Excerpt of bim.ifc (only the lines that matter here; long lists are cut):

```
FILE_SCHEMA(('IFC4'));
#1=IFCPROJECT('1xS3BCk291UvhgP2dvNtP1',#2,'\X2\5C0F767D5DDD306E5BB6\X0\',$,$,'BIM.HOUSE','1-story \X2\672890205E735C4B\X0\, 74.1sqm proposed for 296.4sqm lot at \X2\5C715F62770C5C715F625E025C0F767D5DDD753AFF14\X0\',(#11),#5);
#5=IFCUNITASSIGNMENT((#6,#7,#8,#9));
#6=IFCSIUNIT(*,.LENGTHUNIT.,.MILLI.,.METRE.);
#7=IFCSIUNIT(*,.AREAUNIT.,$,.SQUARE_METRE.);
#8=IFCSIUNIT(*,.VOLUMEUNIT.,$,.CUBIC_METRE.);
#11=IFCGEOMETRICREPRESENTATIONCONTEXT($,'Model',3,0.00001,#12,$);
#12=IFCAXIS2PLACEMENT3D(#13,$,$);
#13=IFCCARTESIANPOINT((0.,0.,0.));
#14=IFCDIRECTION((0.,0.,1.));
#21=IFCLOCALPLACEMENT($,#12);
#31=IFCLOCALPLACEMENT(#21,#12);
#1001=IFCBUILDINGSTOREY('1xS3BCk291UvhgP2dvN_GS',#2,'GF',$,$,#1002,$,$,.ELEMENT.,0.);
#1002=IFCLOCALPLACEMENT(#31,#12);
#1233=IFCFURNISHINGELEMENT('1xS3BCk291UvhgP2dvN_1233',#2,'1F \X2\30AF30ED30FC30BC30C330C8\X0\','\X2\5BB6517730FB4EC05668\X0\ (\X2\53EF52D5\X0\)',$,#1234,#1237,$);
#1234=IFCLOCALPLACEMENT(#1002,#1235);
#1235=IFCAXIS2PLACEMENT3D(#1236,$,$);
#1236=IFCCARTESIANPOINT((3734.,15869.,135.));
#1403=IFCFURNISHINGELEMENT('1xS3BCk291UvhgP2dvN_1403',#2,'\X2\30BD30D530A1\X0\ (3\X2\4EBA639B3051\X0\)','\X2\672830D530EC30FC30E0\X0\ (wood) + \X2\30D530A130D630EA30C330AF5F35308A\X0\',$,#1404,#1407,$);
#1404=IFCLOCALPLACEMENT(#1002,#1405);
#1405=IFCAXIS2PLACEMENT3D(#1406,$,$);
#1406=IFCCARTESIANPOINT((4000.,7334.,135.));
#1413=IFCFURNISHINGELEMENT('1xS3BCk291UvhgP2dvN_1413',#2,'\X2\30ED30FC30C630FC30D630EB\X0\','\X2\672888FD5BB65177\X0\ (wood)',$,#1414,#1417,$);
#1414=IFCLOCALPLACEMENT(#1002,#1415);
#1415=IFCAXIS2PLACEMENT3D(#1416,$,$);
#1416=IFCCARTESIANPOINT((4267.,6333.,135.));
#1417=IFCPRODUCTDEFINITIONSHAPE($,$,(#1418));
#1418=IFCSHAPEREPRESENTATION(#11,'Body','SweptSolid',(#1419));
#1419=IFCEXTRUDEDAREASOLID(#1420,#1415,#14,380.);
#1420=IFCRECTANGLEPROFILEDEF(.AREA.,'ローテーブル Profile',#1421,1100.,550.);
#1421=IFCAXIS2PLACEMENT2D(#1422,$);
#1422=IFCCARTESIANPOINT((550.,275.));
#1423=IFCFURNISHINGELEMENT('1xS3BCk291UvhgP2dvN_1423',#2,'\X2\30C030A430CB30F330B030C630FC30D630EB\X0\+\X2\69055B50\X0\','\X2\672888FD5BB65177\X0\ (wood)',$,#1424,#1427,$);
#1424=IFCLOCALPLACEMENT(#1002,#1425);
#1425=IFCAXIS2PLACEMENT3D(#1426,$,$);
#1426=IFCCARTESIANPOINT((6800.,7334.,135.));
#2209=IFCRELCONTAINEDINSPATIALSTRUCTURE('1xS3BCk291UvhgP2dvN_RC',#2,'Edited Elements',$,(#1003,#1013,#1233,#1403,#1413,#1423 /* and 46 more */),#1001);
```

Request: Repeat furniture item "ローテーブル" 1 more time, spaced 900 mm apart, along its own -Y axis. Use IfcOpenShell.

```python
import ifcopenshell
import ifcopenshell.api.geometry
import ifcopenshell.api.root
import ifcopenshell.util.element
import ifcopenshell.util.placement
import ifcopenshell.util.unit

model = ifcopenshell.open("bim.ifc")
unit_scale = ifcopenshell.util.unit.calculate_unit_scale(model)


def reuse_history(source, copy):
    """copy_class also copies each property set's owner history, people and application; keep the originals."""
    for rel in copy.IsDefinedBy:
        if rel.is_a("IfcRelDefinesByProperties") and (history := rel.RelatingPropertyDefinition.OwnerHistory):
            rel.RelatingPropertyDefinition.OwnerHistory = source.OwnerHistory
            ifcopenshell.util.element.remove_deep2(model, history)


source = model.by_guid("1xS3BCk291UvhgP2dvN_1413")
base = ifcopenshell.util.placement.get_local_placement(source.ObjectPlacement)
step = -base[:3, 1] * 0.9 / unit_scale

for i in range(1, 2):
    copy = ifcopenshell.api.root.copy_class(model, product=source)
    copy.Representation = ifcopenshell.util.element.copy_deep(
        model, source.Representation, exclude=["IfcGeometricRepresentationContext", "IfcRepresentationMap"]
    )
    reuse_history(source, copy)
    matrix = base.copy()
    matrix[:3, 3] += i * step
    print("added at", matrix[:3, 3].round(3) + 0.0)
    ifcopenshell.api.geometry.edit_object_placement(model, product=copy, matrix=matrix, is_si=False)

model.write("bim-out.ifc")
```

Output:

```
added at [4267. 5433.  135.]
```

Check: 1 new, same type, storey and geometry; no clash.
